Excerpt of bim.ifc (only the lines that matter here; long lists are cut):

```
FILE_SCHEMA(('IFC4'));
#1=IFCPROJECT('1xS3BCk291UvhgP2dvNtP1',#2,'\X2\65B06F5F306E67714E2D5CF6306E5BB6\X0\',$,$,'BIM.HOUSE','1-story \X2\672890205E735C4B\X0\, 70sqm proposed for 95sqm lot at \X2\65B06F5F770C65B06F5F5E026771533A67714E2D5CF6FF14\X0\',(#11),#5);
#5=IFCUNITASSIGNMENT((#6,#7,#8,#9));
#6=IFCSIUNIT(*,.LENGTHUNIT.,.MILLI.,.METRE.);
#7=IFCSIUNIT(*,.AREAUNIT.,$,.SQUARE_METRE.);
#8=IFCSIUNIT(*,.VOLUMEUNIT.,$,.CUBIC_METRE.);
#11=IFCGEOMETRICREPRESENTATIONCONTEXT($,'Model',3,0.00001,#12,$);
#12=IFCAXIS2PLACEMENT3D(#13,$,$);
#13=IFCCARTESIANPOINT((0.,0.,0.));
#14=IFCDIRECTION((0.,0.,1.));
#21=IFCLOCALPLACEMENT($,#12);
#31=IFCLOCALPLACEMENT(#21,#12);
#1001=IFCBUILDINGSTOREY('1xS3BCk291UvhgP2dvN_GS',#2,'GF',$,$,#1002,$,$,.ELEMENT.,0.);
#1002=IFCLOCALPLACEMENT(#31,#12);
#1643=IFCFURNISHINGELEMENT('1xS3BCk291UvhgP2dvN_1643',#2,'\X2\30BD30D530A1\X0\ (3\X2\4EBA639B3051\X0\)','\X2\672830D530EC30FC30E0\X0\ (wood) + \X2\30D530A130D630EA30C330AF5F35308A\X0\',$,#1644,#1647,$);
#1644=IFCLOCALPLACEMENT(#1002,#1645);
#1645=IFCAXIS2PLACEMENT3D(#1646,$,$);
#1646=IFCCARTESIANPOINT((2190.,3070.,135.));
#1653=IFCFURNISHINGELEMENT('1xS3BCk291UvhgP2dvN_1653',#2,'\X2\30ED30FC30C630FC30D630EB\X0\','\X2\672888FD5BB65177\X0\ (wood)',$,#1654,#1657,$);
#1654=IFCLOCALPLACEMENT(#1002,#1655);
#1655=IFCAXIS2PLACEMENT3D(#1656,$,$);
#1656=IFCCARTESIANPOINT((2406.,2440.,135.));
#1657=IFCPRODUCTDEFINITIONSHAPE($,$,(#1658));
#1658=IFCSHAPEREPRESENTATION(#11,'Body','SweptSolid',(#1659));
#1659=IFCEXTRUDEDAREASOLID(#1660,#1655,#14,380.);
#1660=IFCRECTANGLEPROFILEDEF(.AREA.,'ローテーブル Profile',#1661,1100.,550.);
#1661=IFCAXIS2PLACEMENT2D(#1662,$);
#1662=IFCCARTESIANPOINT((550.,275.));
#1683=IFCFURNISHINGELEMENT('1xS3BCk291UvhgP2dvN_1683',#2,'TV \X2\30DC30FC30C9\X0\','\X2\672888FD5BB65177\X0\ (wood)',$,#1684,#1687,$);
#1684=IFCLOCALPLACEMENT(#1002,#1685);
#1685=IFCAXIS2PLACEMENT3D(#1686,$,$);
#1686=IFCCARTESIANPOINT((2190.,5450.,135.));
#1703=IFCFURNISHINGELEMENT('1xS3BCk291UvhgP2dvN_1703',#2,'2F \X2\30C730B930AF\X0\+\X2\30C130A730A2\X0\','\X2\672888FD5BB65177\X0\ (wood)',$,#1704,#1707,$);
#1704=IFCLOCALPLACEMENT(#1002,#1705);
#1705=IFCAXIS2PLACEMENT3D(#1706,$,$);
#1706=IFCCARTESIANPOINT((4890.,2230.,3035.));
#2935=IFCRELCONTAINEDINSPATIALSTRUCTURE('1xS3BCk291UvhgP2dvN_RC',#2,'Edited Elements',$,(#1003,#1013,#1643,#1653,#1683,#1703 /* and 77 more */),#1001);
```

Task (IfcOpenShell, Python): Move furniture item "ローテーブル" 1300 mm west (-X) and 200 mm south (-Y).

```python
import ifcopenshell
import ifcopenshell.api.geometry
import ifcopenshell.util.placement

model = ifcopenshell.open("bim.ifc")

item = model.by_guid("1xS3BCk291UvhgP2dvN_1653")
matrix = ifcopenshell.util.placement.get_local_placement(item.ObjectPlacement)
matrix[0, 3] -= 1300.0
matrix[1, 3] -= 200.0
ifcopenshell.api.geometry.edit_object_placement(model, product=item, matrix=matrix, is_si=False)

print(ifcopenshell.util.placement.get_local_placement(item.ObjectPlacement).round(3) + 0.0)

model.write("bim_updated.ifc")
```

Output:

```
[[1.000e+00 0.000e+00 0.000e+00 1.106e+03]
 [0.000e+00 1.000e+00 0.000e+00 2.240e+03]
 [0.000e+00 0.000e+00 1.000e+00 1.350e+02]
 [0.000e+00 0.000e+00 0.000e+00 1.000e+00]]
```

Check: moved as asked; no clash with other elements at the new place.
